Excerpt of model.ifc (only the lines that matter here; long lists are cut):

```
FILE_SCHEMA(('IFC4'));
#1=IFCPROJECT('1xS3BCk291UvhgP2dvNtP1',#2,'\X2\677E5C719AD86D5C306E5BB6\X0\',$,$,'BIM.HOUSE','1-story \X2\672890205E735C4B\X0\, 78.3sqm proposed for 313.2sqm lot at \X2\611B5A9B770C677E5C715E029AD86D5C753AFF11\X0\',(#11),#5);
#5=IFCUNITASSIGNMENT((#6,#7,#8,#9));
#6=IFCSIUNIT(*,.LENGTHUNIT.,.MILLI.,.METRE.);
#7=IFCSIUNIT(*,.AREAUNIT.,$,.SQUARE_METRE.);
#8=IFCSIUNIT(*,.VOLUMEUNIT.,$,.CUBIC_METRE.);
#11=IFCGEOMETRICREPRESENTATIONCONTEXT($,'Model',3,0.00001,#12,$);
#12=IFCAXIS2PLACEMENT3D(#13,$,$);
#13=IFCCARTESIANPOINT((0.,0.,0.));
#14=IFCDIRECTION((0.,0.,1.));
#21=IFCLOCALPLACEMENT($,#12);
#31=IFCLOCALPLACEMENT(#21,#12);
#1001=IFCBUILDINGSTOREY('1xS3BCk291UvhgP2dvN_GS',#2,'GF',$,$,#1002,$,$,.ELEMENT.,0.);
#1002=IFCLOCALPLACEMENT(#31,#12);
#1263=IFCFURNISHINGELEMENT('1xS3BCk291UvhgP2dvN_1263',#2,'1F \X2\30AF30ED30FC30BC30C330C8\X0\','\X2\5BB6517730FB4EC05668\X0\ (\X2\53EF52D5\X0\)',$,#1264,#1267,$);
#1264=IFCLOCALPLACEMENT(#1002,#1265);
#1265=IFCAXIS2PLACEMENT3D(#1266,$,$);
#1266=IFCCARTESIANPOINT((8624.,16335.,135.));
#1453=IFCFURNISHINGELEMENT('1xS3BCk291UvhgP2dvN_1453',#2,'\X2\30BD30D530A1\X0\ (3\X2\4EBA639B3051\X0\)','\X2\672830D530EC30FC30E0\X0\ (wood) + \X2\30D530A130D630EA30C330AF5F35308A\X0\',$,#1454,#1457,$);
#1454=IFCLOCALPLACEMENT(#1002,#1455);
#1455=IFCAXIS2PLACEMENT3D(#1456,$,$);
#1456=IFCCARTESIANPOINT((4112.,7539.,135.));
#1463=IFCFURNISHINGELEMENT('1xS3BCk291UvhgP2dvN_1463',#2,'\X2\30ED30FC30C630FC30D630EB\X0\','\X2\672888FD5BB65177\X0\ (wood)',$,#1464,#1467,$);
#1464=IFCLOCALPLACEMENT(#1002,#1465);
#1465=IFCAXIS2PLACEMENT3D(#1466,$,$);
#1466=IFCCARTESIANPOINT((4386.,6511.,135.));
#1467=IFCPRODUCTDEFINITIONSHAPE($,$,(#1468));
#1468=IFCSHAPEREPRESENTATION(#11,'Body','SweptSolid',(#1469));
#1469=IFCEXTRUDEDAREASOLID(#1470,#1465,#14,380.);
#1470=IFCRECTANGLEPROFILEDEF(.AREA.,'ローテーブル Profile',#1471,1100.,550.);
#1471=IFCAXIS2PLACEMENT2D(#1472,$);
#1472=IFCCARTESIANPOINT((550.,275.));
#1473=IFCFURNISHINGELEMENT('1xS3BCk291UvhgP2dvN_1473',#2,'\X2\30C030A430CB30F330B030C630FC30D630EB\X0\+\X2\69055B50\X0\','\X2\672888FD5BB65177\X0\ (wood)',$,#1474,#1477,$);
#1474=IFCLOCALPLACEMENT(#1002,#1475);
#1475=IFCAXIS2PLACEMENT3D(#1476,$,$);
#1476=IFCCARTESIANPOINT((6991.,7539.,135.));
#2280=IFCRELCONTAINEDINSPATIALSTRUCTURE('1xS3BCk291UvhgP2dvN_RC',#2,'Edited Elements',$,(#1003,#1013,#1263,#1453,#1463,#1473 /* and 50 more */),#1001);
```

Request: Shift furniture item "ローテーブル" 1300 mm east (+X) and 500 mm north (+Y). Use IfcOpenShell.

```python
import ifcopenshell
import ifcopenshell.api.geometry
import ifcopenshell.util.placement

model = ifcopenshell.open("model.ifc")

item = model.by_guid("1xS3BCk291UvhgP2dvN_1463")
matrix = ifcopenshell.util.placement.get_local_placement(item.ObjectPlacement)
matrix[0, 3] += 1300.0
matrix[1, 3] += 500.0
ifcopenshell.api.geometry.edit_object_placement(model, product=item, matrix=matrix, is_si=False)

print(ifcopenshell.util.placement.get_local_placement(item.ObjectPlacement).round(3) + 0.0)

model.write("model_rev.ifc")
```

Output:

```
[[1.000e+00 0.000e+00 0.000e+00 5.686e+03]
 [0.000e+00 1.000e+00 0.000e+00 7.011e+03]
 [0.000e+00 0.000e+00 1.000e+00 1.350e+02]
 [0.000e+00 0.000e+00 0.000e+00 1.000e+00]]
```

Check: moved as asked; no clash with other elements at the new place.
